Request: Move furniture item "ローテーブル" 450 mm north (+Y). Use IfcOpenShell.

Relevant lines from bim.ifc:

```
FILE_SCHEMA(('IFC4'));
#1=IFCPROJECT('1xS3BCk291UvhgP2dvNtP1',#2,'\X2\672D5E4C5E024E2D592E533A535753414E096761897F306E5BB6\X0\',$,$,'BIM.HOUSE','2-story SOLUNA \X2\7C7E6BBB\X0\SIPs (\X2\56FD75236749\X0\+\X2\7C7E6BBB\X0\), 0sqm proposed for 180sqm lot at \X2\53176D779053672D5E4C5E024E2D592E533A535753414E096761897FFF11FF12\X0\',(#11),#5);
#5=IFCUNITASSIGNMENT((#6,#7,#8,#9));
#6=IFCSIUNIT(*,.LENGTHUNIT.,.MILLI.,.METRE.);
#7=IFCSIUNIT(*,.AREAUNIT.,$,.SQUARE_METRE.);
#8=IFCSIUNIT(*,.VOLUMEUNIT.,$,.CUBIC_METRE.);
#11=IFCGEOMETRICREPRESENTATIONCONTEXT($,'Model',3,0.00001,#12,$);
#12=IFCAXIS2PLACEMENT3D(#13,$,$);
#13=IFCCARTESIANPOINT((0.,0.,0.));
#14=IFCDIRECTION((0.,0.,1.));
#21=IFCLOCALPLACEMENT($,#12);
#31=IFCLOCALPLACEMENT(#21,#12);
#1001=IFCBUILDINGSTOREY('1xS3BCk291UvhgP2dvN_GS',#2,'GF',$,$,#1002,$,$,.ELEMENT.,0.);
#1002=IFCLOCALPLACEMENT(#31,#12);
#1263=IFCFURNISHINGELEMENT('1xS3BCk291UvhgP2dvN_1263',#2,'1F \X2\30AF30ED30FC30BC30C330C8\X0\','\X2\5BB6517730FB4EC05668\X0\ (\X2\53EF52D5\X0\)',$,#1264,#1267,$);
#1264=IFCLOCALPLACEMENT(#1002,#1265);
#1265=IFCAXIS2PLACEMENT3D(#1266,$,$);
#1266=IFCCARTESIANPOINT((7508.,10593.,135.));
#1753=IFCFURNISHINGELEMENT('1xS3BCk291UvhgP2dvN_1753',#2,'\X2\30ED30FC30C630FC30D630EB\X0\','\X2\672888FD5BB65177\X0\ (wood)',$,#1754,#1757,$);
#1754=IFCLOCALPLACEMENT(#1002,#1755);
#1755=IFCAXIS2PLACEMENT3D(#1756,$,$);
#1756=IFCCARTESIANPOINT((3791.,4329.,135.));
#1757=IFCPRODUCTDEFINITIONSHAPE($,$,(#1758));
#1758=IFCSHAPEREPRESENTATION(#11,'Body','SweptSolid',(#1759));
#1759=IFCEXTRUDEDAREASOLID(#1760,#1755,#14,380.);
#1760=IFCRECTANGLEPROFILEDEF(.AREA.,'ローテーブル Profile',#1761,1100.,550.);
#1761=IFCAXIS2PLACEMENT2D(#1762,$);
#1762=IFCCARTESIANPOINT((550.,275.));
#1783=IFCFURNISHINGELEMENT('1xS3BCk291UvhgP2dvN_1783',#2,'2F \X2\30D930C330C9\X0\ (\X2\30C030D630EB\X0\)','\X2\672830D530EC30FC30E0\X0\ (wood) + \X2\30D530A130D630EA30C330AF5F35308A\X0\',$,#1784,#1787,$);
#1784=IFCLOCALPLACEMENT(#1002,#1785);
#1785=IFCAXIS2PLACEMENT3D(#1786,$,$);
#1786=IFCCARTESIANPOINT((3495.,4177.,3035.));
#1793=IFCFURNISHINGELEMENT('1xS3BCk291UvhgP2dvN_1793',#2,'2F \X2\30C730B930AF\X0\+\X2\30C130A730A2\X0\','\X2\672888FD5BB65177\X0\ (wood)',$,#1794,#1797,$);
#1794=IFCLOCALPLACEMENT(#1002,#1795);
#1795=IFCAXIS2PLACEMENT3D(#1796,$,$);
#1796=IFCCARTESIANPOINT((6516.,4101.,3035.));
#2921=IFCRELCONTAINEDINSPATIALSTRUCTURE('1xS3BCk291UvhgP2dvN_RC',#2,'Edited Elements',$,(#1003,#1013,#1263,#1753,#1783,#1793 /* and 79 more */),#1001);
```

```python
import ifcopenshell
import ifcopenshell.api.geometry
import ifcopenshell.util.placement
import ifcopenshell.util.unit

model = ifcopenshell.open("bim.ifc")
unit_scale = ifcopenshell.util.unit.calculate_unit_scale(model)

item = model.by_id(1753)
matrix = ifcopenshell.util.placement.get_local_placement(item.ObjectPlacement)
matrix[1, 3] += 0.45 / unit_scale
ifcopenshell.api.geometry.edit_object_placement(model, product=item, matrix=matrix, is_si=False)

print(ifcopenshell.util.placement.get_local_placement(item.ObjectPlacement).round(3) + 0.0)

model.write("bim_v2.ifc")
```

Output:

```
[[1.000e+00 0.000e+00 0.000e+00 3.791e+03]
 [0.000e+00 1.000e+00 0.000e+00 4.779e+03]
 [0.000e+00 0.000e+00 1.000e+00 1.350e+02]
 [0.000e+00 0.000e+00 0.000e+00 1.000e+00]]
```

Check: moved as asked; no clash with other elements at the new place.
